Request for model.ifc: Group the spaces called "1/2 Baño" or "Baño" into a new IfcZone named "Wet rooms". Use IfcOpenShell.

First a look at what the model holds.

```python
import ifcopenshell

model = ifcopenshell.open("model.ifc")
print(model.schema)
seen = {}
for space in model.by_type("IfcSpace"):
    seen[space.LongName] = seen.get(space.LongName, 0) + 1
for name, count in sorted(seen.items(), key=str):
    print(count, "x", name)
print("zones:", [z.Name for z in model.by_type("IfcZone")][:20])
```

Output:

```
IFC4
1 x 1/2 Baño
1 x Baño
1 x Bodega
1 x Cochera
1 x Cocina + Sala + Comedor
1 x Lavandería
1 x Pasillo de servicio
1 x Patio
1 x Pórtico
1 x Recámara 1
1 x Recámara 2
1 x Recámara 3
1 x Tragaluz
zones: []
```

```python
import ifcopenshell
import ifcopenshell.api.group
import ifcopenshell.api.root

model = ifcopenshell.open("model.ifc")

names = {"1/2 Baño", "Baño"}
spaces = [s for s in model.by_type("IfcSpace") if s.LongName in names]

zone = ifcopenshell.api.root.create_entity(model, ifc_class="IfcZone", name="Wet rooms")
ifcopenshell.api.group.assign_group(model, products=spaces, group=zone)
print(len(spaces), "spaces in", zone.Name)

model.write("model_rev.ifc")
```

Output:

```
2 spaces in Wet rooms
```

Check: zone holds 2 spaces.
